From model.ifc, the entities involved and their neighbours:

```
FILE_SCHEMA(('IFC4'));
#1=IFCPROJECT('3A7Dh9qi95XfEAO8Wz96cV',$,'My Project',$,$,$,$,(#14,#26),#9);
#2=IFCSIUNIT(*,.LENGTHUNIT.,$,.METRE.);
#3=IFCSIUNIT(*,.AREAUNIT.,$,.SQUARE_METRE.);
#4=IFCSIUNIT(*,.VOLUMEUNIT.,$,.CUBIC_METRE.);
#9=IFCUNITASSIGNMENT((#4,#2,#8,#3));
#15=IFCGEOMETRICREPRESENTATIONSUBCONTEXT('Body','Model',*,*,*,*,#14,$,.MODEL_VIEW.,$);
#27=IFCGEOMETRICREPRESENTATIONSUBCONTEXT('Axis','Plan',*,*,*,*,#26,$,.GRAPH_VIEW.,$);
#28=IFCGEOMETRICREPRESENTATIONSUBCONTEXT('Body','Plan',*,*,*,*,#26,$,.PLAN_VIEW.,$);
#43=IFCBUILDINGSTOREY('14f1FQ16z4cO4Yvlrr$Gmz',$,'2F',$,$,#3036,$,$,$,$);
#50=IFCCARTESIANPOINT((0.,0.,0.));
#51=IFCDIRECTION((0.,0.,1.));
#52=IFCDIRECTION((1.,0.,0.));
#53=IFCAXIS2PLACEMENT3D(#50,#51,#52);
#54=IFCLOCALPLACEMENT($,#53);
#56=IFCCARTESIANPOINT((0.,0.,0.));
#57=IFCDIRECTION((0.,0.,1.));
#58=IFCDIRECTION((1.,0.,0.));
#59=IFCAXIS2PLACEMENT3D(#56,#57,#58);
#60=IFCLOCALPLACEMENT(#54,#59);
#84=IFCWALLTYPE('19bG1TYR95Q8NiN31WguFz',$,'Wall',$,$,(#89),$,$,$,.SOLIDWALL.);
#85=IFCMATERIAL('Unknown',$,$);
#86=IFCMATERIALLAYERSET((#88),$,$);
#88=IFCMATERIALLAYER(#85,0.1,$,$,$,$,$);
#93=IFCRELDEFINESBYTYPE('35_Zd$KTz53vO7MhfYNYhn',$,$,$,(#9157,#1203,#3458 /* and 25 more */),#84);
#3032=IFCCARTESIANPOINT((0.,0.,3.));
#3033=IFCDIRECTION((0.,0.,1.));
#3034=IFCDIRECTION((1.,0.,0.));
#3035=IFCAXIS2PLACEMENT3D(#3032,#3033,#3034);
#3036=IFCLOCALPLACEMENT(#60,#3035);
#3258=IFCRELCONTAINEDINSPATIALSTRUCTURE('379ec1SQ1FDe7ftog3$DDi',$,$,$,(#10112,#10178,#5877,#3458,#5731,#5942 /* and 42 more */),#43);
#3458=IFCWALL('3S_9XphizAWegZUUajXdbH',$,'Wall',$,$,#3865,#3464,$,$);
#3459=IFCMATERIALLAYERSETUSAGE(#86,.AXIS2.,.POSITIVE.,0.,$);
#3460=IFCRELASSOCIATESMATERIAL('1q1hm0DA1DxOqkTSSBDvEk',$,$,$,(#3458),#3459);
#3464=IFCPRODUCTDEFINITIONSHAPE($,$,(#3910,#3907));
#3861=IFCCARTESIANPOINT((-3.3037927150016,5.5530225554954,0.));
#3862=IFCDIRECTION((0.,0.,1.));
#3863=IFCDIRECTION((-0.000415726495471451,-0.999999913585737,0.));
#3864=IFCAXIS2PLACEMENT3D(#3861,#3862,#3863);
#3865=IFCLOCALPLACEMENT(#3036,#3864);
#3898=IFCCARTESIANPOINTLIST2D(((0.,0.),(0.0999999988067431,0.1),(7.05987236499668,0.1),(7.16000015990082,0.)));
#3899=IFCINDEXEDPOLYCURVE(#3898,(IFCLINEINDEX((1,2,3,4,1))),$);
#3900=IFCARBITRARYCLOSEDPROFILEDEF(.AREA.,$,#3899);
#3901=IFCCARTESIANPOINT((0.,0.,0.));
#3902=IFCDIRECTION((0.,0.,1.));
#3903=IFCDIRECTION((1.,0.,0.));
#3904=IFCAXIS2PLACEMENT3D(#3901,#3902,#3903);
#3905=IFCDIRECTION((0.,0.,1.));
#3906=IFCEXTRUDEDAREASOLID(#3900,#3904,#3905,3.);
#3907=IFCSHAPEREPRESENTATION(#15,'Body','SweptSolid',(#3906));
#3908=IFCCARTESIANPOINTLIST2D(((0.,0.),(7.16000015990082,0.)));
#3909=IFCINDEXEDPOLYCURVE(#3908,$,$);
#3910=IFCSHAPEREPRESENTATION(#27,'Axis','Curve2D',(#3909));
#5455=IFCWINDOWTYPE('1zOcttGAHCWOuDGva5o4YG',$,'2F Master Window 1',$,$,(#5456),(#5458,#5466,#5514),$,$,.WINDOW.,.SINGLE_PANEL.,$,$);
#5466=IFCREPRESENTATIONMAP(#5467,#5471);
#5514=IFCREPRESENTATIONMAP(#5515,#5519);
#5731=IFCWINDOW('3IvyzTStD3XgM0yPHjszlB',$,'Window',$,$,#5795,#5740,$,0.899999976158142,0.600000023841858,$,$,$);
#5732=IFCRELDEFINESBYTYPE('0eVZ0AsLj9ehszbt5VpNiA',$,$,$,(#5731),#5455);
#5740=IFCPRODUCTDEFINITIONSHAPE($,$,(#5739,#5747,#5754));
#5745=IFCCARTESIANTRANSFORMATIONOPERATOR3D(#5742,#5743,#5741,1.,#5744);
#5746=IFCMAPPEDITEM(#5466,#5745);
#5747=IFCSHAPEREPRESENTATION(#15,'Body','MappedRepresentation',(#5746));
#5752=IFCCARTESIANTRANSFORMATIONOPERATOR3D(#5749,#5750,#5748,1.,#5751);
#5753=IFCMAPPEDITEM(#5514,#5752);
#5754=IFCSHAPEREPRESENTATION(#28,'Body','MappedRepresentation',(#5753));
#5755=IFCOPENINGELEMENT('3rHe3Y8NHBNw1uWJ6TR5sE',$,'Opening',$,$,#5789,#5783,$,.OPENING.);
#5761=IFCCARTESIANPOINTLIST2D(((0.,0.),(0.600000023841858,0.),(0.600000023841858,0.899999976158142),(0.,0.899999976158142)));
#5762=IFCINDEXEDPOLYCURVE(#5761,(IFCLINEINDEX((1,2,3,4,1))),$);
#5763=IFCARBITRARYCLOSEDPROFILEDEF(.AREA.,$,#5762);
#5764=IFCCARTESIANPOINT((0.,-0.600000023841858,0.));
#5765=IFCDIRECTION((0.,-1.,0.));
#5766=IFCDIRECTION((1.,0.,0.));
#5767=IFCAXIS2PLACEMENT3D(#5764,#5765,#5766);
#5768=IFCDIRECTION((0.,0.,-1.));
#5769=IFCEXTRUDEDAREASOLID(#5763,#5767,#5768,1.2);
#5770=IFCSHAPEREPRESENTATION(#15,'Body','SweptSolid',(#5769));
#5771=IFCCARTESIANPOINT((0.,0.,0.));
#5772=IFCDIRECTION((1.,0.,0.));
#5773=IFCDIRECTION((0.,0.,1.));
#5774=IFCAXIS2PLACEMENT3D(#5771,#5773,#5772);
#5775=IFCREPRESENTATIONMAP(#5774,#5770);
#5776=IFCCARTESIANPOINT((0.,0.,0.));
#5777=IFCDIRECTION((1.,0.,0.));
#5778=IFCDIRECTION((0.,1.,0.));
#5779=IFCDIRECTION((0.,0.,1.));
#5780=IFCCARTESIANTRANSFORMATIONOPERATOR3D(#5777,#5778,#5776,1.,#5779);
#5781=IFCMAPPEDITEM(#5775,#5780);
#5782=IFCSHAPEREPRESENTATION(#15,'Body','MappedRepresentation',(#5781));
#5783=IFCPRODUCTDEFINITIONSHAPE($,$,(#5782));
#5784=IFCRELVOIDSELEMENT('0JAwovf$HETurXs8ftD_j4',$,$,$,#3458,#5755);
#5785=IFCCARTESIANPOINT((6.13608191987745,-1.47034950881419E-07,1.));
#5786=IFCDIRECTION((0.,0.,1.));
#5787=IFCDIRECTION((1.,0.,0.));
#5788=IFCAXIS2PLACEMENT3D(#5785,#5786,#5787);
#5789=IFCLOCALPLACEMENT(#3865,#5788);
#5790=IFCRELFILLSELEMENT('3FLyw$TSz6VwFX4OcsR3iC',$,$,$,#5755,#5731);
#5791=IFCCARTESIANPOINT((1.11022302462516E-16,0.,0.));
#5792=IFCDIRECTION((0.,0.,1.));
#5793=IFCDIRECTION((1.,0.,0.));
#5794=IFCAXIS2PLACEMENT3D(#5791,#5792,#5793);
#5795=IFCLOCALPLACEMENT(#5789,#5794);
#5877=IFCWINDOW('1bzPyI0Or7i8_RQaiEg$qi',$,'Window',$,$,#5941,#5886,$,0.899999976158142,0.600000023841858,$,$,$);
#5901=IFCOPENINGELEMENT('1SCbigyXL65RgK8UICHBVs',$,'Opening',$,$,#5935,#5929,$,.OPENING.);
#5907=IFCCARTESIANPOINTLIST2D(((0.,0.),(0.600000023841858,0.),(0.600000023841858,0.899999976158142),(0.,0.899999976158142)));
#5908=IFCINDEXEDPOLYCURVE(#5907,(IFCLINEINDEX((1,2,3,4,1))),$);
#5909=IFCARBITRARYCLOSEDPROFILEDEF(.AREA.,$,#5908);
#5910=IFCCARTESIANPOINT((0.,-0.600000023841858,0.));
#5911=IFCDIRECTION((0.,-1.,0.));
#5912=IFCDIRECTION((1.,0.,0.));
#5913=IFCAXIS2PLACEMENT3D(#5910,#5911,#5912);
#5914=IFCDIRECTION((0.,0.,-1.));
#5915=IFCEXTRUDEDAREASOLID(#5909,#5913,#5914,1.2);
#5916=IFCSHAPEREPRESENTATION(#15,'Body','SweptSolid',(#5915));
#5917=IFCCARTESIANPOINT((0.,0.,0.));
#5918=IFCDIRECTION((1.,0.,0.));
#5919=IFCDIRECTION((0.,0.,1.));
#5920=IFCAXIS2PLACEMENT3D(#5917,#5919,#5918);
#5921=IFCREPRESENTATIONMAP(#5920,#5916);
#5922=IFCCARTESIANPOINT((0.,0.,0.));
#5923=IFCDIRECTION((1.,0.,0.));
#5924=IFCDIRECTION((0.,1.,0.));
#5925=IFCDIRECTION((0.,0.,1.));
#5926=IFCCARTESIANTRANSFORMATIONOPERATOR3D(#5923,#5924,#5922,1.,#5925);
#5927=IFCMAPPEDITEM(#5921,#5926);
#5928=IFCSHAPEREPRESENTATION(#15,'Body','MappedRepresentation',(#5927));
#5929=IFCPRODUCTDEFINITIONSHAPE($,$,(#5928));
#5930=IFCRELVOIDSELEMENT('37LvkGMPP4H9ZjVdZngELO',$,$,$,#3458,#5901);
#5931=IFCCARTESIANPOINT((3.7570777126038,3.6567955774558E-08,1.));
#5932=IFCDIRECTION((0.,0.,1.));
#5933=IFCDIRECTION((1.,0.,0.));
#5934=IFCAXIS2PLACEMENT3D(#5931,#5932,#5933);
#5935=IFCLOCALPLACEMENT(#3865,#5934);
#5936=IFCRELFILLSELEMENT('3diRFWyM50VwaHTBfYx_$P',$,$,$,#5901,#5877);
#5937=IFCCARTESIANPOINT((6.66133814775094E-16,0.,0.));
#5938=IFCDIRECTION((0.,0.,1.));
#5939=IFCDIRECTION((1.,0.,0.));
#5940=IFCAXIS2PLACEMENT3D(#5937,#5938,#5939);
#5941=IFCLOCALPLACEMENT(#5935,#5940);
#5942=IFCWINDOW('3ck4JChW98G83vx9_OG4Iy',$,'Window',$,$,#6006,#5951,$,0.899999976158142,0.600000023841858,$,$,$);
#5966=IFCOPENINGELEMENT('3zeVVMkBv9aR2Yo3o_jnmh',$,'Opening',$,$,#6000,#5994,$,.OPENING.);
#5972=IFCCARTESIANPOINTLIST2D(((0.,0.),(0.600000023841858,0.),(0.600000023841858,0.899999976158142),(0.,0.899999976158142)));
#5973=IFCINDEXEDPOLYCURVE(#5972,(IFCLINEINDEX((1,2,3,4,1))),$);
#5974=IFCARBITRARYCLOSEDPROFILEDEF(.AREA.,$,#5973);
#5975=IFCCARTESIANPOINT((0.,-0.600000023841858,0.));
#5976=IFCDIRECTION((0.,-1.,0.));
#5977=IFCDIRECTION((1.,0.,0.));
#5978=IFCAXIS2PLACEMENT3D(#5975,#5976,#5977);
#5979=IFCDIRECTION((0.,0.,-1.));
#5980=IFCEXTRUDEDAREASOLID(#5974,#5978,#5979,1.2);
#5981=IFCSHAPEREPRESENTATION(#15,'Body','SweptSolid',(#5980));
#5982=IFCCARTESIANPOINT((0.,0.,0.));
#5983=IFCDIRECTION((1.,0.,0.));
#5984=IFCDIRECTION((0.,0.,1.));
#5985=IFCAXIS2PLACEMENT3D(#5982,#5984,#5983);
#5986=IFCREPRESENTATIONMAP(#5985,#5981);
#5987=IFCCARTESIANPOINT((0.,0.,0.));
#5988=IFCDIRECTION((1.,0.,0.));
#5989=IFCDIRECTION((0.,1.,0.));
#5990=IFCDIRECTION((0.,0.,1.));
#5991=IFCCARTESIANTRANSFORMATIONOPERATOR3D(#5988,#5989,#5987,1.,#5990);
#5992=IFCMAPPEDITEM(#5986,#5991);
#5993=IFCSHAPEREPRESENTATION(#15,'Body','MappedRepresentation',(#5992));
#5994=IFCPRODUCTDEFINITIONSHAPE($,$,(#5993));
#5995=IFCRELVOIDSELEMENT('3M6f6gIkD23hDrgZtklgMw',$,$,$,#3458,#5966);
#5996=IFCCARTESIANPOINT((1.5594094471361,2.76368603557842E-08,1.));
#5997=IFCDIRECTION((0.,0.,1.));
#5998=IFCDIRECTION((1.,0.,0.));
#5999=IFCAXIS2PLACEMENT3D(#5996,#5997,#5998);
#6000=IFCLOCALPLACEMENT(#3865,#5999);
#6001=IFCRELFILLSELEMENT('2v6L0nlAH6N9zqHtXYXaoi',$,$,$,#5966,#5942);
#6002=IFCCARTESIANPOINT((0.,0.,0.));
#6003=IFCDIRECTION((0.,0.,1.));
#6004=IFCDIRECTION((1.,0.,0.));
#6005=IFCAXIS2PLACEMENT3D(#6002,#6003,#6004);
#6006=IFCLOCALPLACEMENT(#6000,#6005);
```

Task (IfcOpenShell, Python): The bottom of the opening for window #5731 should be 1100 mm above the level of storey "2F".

```python
import numpy as np
import ifcopenshell
import ifcopenshell.api.geometry
import ifcopenshell.geom
import ifcopenshell.util.element
import ifcopenshell.util.placement
import ifcopenshell.util.shape
import ifcopenshell.util.unit

model = ifcopenshell.open("model.ifc")
unit_scale = ifcopenshell.util.unit.calculate_unit_scale(model)

window = model.by_guid("3IvyzTStD3XgM0yPHjszlB")
opening = window.FillsVoids[0].RelatingOpeningElement
storey = ifcopenshell.util.element.get_container(window, ifc_class="IfcBuildingStorey")
level = ifcopenshell.util.placement.get_local_placement(storey.ObjectPlacement)[2, 3]

# The opening's origin need not be at the sill, so measure its lowest point.
shape = ifcopenshell.geom.create_shape(ifcopenshell.geom.settings(), opening)
bottom = ifcopenshell.util.shape.get_shape_bottom_elevation(shape, shape.geometry) / unit_scale
dz = level + 1.1 - bottom

shift = np.array([0.0, 0.0, dz])
# The window is placed relative to its opening, so it follows when the opening moves.
matrix = ifcopenshell.util.placement.get_local_placement(opening.ObjectPlacement)
matrix[:3, 3] += shift
ifcopenshell.api.geometry.edit_object_placement(
    model, product=opening, matrix=matrix, is_si=False, should_transform_children=True
)

print(f"moved by {dz * unit_scale:+.3f} m")

model.write("model_updated.ifc")
```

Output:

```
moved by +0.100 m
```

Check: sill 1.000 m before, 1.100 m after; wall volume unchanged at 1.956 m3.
